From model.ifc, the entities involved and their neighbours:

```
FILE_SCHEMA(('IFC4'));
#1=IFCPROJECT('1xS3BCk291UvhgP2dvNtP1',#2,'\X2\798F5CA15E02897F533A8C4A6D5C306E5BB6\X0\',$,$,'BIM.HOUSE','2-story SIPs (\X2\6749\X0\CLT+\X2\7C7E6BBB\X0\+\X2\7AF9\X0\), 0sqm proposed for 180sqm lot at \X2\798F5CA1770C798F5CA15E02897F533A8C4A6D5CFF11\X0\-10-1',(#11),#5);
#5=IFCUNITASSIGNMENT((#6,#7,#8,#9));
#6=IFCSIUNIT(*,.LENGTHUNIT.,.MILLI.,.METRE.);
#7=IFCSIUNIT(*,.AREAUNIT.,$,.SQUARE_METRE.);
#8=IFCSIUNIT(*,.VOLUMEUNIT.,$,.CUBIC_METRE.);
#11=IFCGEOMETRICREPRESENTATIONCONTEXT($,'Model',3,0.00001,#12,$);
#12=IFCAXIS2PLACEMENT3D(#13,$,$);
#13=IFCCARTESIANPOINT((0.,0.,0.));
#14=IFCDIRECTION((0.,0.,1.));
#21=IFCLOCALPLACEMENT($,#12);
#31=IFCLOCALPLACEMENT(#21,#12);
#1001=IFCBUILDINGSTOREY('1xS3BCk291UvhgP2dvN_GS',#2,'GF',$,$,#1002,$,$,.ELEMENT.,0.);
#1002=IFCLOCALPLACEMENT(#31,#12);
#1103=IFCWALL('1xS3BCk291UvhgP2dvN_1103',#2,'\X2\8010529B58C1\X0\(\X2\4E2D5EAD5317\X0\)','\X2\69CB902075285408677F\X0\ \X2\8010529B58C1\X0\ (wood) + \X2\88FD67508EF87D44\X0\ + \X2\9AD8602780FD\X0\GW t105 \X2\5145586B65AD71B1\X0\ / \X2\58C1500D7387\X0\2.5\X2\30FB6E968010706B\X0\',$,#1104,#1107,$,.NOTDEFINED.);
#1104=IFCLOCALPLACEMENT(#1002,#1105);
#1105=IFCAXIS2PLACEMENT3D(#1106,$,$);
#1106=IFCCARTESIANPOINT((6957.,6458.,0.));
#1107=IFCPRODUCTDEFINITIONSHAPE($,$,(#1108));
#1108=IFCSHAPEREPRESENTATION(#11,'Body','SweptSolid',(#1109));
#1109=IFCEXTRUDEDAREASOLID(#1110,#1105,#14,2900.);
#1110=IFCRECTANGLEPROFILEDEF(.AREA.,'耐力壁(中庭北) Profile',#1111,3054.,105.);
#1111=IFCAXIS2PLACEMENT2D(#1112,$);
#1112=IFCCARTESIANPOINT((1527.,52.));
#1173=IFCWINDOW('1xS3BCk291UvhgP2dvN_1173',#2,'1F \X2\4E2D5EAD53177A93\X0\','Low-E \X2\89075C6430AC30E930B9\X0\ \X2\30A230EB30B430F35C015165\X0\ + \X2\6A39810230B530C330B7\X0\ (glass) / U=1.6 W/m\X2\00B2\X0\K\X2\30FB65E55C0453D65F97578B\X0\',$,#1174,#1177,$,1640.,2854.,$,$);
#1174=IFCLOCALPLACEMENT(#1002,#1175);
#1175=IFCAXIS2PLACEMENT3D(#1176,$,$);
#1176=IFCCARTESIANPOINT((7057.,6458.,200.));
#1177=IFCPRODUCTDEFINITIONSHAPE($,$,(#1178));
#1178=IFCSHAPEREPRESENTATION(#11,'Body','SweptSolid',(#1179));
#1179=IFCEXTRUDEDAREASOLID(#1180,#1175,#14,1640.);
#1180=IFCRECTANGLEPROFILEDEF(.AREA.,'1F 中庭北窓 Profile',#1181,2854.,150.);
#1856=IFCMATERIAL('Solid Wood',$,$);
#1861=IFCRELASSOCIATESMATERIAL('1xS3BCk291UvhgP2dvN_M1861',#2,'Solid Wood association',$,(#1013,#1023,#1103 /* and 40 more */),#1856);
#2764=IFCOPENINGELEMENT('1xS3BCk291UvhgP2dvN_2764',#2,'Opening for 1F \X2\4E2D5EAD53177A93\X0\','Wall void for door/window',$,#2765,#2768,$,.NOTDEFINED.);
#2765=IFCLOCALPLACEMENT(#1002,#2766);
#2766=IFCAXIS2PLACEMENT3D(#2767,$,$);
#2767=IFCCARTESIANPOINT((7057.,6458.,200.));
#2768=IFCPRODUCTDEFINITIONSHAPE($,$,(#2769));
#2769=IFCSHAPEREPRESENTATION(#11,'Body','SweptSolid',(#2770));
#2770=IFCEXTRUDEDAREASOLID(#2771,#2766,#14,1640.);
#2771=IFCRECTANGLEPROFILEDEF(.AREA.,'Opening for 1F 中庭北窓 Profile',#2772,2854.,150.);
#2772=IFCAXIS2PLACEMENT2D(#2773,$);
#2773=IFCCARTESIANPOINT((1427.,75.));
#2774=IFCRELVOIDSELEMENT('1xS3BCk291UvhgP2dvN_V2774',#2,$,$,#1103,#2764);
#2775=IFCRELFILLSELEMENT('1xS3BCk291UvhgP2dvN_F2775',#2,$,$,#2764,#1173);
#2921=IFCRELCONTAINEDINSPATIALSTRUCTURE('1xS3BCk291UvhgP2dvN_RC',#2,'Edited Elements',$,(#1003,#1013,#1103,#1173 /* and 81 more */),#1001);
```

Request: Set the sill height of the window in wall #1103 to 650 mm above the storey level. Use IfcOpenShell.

```python
import numpy as np
import ifcopenshell
import ifcopenshell.api.geometry
import ifcopenshell.geom
import ifcopenshell.util.element
import ifcopenshell.util.placement
import ifcopenshell.util.shape
import ifcopenshell.util.unit

model = ifcopenshell.open("model.ifc")
unit_scale = ifcopenshell.util.unit.calculate_unit_scale(model)

window = model.by_id(1173)
opening = window.FillsVoids[0].RelatingOpeningElement
storey = ifcopenshell.util.element.get_container(window, ifc_class="IfcBuildingStorey")
level = ifcopenshell.util.placement.get_local_placement(storey.ObjectPlacement)[2, 3]

# The opening's origin need not be at the sill, so measure its lowest point.
shape = ifcopenshell.geom.create_shape(ifcopenshell.geom.settings(), opening)
bottom = ifcopenshell.util.shape.get_shape_bottom_elevation(shape, shape.geometry) / unit_scale
dz = level + 650.0 - bottom

shift = np.array([0.0, 0.0, dz])
# The window is not placed relative to its opening, so move both.
for product in (opening, window):
    matrix = ifcopenshell.util.placement.get_local_placement(product.ObjectPlacement)
    matrix[:3, 3] += shift
    ifcopenshell.api.geometry.edit_object_placement(model, product=product, matrix=matrix, is_si=False)

print(f"moved by {dz * unit_scale:+.3f} m")

model.write("model-out.ifc")
```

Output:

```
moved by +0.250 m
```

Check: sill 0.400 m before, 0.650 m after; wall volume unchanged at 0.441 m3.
